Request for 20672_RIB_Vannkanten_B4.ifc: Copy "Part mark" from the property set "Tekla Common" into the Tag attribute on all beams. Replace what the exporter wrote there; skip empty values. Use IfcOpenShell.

First a look at what the model holds.

```python
import ifcopenshell
import ifcopenshell.util.element

model = ifcopenshell.open("20672_RIB_Vannkanten_B4.ifc")
print(model.schema)
beams = model.by_type("IfcBeam")
print(len(beams), "beams")
for e in beams[:8]:
    source = ifcopenshell.util.element.get_pset(e, "Tekla Common", "Part mark")
    target = e.Tag
    print(e.id(), repr(source), repr(target), sep=" | ")
```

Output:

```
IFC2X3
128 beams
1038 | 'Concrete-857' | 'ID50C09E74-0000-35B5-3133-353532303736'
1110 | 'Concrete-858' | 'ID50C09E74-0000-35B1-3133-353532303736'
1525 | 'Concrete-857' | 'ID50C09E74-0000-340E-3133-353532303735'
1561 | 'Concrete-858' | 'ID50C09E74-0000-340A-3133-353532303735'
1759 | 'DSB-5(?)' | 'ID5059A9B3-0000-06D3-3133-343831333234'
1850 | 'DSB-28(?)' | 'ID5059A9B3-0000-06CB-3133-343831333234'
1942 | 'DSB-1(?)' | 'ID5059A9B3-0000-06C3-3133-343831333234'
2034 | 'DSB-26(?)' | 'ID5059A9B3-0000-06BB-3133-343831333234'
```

```python
import ifcopenshell
import ifcopenshell.util.element

model = ifcopenshell.open("20672_RIB_Vannkanten_B4.ifc")

count = 0
for e in model.by_type("IfcBeam"):
    value = ifcopenshell.util.element.get_pset(e, "Tekla Common", "Part mark")
    current = e.Tag
    if not value or not value.strip() or current == value:
        continue
    e.Tag = value
    count += 1

print(count, "beams updated")

model.write("20672_RIB_Vannkanten_B4_v2.ifc")
```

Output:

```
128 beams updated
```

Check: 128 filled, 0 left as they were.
